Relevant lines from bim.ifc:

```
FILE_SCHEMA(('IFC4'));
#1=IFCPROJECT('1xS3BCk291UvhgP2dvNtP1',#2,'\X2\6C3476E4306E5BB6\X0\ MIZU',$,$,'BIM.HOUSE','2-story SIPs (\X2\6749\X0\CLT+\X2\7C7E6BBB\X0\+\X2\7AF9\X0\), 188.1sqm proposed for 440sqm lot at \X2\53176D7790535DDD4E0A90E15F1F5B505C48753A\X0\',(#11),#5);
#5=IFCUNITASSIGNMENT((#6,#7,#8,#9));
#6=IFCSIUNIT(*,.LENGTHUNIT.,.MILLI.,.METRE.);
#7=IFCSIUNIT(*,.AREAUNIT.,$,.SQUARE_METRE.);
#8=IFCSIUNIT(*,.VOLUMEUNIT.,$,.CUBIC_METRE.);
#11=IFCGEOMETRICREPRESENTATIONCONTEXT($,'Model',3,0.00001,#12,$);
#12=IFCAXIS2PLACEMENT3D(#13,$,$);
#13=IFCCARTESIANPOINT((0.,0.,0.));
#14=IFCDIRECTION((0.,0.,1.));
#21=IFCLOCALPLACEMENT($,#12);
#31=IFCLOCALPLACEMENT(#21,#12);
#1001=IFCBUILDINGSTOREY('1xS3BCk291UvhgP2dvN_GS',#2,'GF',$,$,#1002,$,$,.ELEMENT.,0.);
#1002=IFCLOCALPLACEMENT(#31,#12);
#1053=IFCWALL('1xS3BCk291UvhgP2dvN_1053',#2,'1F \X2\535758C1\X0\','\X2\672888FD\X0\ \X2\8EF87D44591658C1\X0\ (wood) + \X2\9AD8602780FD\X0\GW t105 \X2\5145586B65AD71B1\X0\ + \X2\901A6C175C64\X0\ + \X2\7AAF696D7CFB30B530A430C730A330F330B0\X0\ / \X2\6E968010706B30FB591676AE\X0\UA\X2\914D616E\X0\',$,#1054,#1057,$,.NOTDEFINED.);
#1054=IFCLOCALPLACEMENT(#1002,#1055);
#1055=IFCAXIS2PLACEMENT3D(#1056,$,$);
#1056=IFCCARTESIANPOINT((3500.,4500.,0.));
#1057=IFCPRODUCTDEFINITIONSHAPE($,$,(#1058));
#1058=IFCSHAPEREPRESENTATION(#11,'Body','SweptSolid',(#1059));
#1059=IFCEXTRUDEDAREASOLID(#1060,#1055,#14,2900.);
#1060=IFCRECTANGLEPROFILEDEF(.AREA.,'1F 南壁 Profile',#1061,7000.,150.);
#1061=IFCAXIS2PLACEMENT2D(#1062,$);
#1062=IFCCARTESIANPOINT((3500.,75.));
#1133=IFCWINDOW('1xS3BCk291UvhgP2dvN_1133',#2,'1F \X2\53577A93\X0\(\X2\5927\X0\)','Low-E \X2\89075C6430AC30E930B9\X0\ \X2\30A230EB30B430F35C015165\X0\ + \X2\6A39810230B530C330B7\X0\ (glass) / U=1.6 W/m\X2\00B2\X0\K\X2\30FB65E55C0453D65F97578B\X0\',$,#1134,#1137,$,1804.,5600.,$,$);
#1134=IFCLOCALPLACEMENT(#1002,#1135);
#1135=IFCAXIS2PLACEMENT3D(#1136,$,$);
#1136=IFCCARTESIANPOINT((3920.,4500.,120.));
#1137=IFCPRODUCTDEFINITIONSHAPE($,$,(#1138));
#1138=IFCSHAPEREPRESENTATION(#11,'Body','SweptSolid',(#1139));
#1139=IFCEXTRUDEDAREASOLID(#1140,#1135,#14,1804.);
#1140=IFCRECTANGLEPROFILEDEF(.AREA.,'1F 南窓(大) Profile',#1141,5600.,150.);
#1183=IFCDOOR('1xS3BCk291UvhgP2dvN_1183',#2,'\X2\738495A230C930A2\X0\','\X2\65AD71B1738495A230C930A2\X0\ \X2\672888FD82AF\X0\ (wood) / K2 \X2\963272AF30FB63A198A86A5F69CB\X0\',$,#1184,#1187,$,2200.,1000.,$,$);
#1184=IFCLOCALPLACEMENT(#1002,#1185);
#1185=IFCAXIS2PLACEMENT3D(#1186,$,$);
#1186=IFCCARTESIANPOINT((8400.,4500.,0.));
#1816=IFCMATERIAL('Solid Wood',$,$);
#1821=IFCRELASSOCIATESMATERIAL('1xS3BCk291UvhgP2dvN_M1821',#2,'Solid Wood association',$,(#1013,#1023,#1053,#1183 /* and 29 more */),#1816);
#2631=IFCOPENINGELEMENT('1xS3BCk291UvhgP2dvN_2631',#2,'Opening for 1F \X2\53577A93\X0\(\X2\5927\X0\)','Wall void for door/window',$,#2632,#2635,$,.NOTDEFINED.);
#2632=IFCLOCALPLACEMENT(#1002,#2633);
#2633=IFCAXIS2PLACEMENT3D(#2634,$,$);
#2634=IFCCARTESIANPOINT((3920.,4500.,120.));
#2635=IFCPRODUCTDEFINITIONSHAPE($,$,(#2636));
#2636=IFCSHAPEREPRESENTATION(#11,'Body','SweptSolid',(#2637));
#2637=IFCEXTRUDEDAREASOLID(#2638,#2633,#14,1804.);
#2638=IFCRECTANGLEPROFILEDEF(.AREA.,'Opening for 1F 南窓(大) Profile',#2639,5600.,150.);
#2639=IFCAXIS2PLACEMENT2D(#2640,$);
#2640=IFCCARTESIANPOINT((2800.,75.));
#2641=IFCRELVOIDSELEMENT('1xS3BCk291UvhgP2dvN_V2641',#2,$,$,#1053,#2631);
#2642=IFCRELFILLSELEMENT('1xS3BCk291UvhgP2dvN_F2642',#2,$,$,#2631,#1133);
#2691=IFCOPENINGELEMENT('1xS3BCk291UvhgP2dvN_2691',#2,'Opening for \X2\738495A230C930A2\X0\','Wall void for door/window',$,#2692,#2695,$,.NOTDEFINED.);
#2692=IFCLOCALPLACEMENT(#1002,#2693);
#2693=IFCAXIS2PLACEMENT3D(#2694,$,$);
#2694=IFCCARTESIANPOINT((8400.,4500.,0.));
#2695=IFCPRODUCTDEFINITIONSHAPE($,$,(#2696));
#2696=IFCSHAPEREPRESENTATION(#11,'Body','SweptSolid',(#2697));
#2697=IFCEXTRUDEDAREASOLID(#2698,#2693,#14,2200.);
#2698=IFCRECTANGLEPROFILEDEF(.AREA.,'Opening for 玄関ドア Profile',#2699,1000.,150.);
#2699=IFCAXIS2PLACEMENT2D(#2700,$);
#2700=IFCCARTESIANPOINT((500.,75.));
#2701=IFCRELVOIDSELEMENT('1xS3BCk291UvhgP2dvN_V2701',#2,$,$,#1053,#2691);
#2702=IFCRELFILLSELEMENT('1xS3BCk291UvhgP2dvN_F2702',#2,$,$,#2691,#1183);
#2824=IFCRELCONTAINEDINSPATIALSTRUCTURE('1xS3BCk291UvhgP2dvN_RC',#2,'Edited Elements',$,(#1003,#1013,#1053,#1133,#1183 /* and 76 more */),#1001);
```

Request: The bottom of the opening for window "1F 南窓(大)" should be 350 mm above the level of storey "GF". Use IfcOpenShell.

```python
import numpy as np
import ifcopenshell
import ifcopenshell.api.geometry
import ifcopenshell.geom
import ifcopenshell.util.element
import ifcopenshell.util.placement
import ifcopenshell.util.shape
import ifcopenshell.util.unit

model = ifcopenshell.open("bim.ifc")
unit_scale = ifcopenshell.util.unit.calculate_unit_scale(model)

window = model.by_id(1133)
opening = window.FillsVoids[0].RelatingOpeningElement
storey = ifcopenshell.util.element.get_container(window, ifc_class="IfcBuildingStorey")
level = ifcopenshell.util.placement.get_local_placement(storey.ObjectPlacement)[2, 3]

# The opening's origin need not be at the sill, so measure its lowest point.
shape = ifcopenshell.geom.create_shape(ifcopenshell.geom.settings(), opening)
bottom = ifcopenshell.util.shape.get_shape_bottom_elevation(shape, shape.geometry) / unit_scale
dz = level + 350.0 - bottom

shift = np.array([0.0, 0.0, dz])
# The window is not placed relative to its opening, so move both.
for product in (opening, window):
    matrix = ifcopenshell.util.placement.get_local_placement(product.ObjectPlacement)
    matrix[:3, 3] += shift
    ifcopenshell.api.geometry.edit_object_placement(model, product=product, matrix=matrix, is_si=False)

print(f"moved by {dz * unit_scale:+.3f} m")

model.write("bim_v2.ifc")
```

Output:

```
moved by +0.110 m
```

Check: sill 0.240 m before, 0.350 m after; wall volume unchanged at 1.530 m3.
